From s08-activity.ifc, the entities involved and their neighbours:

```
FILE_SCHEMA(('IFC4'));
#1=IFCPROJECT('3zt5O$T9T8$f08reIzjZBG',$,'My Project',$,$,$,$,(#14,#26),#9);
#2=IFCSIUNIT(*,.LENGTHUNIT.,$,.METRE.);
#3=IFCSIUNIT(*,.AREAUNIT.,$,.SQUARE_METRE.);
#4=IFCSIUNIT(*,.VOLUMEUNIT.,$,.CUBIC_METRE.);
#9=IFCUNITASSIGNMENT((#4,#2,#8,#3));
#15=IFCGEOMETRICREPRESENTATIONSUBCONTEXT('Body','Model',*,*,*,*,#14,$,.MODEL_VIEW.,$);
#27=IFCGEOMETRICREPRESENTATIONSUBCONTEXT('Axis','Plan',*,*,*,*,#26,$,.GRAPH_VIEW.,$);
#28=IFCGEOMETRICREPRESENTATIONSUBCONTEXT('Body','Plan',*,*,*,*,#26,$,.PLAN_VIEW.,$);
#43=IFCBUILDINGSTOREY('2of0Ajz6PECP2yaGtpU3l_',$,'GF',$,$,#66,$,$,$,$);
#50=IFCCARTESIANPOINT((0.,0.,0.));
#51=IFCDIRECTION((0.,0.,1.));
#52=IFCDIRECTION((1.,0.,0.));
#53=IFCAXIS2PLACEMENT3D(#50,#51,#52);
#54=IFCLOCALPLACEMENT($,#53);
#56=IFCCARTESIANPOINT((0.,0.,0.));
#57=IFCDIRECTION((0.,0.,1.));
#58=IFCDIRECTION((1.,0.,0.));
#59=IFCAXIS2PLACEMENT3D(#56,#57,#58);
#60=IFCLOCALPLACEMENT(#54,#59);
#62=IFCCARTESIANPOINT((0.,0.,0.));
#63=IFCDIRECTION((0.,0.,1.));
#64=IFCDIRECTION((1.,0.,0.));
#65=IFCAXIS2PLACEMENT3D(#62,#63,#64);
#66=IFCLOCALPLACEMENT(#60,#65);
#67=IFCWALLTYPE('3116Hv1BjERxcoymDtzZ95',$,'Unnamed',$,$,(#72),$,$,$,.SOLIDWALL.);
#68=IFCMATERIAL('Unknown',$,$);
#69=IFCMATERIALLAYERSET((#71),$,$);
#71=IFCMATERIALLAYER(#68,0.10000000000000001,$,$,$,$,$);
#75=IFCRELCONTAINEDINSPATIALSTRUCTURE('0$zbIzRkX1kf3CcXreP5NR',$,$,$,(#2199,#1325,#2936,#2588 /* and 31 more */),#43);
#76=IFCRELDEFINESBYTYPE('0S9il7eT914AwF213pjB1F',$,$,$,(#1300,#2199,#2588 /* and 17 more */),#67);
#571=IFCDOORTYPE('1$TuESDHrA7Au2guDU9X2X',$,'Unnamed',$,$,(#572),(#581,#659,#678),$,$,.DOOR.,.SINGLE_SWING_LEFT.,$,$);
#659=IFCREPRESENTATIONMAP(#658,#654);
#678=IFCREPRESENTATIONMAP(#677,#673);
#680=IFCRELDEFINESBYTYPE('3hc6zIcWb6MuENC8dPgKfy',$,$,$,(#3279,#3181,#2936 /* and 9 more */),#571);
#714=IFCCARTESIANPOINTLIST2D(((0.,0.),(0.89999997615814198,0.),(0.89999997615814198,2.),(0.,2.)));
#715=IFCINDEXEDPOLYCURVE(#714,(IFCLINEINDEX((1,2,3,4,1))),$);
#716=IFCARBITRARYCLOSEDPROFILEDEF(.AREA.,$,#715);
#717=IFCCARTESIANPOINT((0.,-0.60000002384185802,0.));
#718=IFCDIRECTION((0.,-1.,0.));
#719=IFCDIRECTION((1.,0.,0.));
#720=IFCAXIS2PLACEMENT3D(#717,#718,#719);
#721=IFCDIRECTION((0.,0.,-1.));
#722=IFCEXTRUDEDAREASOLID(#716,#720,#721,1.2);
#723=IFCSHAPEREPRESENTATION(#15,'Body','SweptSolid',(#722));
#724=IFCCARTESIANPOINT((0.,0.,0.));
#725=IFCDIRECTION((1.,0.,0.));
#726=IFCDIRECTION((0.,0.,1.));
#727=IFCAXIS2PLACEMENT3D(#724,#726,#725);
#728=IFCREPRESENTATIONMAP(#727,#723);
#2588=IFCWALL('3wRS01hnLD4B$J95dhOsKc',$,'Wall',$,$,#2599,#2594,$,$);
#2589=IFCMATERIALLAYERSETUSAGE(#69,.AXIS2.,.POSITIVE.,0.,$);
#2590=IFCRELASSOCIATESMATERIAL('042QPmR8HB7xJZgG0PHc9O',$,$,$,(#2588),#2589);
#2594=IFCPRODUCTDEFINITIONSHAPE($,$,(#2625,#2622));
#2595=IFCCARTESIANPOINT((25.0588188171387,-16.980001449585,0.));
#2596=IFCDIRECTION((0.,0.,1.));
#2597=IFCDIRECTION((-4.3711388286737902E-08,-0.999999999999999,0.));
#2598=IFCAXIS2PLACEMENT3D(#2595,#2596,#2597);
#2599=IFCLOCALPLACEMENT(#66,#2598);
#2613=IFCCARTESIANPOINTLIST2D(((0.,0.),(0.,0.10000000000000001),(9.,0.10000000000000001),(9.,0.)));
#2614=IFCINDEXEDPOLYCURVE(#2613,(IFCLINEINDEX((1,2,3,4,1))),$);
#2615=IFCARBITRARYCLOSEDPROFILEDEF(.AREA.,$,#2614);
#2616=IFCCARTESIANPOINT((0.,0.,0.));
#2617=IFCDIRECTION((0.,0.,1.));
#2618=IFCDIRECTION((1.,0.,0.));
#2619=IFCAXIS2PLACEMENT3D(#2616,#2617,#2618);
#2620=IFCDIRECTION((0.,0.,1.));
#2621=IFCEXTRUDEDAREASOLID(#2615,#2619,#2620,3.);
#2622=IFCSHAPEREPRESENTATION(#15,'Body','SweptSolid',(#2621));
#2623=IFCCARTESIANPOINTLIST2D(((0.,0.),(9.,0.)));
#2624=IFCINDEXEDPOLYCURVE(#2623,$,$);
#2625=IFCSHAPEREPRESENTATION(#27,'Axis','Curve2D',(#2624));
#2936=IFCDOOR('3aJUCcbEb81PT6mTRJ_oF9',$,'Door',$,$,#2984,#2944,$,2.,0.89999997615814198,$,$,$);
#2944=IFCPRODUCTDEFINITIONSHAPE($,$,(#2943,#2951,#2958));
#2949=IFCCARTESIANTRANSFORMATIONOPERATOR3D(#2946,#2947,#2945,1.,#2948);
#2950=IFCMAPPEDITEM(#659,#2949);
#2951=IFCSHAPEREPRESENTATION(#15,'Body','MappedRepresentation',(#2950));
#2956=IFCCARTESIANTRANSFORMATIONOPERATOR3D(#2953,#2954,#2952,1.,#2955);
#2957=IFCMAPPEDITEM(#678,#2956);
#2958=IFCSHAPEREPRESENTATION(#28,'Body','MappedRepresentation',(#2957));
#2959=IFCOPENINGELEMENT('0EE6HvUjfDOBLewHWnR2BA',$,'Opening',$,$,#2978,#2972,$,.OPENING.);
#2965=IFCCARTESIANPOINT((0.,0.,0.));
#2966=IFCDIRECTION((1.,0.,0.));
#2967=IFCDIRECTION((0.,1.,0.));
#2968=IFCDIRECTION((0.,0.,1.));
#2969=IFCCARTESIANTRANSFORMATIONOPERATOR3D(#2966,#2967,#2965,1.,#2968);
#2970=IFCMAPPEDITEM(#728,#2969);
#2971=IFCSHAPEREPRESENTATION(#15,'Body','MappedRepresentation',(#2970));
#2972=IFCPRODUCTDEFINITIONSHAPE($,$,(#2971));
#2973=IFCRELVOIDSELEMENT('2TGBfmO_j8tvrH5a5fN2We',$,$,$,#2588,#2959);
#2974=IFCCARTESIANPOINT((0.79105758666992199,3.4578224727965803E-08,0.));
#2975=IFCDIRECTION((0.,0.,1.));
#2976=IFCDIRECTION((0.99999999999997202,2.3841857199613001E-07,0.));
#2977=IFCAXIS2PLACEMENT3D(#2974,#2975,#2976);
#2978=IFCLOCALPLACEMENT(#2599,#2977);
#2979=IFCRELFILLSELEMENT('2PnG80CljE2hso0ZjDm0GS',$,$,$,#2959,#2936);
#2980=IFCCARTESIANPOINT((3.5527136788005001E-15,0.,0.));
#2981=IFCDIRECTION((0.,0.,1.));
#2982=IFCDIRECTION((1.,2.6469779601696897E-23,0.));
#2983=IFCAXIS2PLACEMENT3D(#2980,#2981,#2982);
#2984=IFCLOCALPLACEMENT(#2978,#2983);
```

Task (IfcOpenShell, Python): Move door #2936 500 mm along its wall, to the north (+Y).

```python
import ifcopenshell
import ifcopenshell.api.geometry
import ifcopenshell.util.placement

model = ifcopenshell.open("s08-activity.ifc")

door = model.by_guid("3aJUCcbEb81PT6mTRJ_oF9")
opening = door.FillsVoids[0].RelatingOpeningElement
wall = opening.VoidsElements[0].RelatingBuildingElement

wall_matrix = ifcopenshell.util.placement.get_local_placement(wall.ObjectPlacement)
shift = wall_matrix[:3, 0] * -0.5
before = ifcopenshell.util.placement.get_local_placement(door.ObjectPlacement)[:3, 3].copy()

# The door is placed relative to its opening, so it follows when the opening moves.
matrix = ifcopenshell.util.placement.get_local_placement(opening.ObjectPlacement)
matrix[:3, 3] += shift
ifcopenshell.api.geometry.edit_object_placement(
    model, product=opening, matrix=matrix, is_si=False, should_transform_children=True
)

after = ifcopenshell.util.placement.get_local_placement(door.ObjectPlacement)[:3, 3]
print("door moved by", (after - before).round(3) + 0.0)

model.write("s08-activity_updated.ifc")
```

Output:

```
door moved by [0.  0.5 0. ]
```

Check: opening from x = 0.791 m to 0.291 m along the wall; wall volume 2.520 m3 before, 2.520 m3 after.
